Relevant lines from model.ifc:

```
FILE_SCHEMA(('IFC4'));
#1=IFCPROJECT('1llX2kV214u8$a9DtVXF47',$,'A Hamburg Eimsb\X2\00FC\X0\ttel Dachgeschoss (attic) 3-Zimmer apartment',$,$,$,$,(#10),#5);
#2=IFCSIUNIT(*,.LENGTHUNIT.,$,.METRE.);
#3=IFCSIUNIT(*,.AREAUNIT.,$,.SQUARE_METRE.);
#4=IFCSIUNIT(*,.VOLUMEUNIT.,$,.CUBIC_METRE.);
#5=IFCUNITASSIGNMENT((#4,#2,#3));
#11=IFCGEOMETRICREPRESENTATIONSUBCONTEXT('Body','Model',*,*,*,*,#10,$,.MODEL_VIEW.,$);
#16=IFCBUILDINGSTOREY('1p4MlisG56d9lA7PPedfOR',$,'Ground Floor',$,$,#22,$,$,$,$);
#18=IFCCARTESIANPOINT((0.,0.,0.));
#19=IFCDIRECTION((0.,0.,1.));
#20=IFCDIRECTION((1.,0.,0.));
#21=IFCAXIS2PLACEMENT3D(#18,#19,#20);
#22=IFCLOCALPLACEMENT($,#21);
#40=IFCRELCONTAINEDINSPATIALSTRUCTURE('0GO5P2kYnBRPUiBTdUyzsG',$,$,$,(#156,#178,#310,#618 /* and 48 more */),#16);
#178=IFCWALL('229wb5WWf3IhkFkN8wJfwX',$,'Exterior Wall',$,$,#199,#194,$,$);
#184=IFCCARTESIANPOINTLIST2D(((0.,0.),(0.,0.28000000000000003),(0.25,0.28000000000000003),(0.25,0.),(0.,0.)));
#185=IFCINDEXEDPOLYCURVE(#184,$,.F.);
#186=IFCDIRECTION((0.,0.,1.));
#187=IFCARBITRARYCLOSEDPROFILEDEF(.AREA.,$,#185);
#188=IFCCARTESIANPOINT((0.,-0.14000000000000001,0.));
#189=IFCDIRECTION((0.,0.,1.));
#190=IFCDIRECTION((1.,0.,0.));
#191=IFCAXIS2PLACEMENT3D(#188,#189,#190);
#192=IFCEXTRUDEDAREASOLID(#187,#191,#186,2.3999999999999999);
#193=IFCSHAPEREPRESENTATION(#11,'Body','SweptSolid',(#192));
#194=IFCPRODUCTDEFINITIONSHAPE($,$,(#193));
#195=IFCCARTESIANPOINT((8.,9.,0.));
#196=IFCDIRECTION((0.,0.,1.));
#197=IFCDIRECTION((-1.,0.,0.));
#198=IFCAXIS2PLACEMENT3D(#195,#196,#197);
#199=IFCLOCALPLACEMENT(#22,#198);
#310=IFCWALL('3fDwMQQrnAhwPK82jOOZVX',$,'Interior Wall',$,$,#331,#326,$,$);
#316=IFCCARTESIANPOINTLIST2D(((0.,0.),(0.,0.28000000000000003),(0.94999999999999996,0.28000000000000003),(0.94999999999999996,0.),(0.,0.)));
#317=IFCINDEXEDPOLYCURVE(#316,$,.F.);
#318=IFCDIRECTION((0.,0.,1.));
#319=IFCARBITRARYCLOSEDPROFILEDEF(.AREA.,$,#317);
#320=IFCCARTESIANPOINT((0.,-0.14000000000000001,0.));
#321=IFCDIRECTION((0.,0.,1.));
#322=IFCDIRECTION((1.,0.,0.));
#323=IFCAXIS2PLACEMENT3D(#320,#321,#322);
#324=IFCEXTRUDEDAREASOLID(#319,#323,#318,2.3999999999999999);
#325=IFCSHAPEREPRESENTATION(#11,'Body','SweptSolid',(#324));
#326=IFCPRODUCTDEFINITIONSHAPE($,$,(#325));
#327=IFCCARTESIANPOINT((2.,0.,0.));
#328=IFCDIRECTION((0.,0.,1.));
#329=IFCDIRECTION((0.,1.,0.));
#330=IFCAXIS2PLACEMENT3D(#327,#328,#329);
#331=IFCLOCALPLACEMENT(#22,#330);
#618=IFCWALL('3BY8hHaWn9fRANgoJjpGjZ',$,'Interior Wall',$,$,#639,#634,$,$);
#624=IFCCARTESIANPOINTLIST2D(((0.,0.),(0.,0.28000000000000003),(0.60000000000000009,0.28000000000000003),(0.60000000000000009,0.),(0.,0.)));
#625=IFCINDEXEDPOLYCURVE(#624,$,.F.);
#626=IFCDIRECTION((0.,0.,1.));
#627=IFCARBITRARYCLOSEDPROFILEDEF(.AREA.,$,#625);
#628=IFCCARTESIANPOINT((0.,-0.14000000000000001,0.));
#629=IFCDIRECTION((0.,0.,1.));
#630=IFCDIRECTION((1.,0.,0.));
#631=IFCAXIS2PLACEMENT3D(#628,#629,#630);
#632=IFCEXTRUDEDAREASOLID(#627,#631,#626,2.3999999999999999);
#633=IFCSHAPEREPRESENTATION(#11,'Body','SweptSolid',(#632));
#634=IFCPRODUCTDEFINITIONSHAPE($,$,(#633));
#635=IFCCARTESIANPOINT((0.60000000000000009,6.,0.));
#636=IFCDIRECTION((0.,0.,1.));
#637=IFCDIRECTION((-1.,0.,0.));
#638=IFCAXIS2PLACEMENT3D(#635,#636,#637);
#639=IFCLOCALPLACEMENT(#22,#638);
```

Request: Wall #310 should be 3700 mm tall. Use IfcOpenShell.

```python
import ifcopenshell
import ifcopenshell.geom
import ifcopenshell.util.representation
import ifcopenshell.util.shape
import ifcopenshell.util.unit

model = ifcopenshell.open("model.ifc")
unit_scale = ifcopenshell.util.unit.calculate_unit_scale(model)
settings = ifcopenshell.geom.settings()


def volume(element):
    """Net volume in cubic metres, openings subtracted."""
    shape = ifcopenshell.geom.create_shape(settings, element)
    return ifcopenshell.util.shape.get_volume(shape.geometry)


wall = model.by_guid("3fDwMQQrnAhwPK82jOOZVX")
before = volume(wall)

body = ifcopenshell.util.representation.get_representation(wall, "Model", "Body")
solid = body.Items[0]
old_height = solid.Depth
solid.Depth = 3.7 / unit_scale
after = volume(wall)

print(f"height {old_height:g} -> {solid.Depth:g}, volume {before:.3f} -> {after:.3f} m3")

model.write("model_updated.ifc")
```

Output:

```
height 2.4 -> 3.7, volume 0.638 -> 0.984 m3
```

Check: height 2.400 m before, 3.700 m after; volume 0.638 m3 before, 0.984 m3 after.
